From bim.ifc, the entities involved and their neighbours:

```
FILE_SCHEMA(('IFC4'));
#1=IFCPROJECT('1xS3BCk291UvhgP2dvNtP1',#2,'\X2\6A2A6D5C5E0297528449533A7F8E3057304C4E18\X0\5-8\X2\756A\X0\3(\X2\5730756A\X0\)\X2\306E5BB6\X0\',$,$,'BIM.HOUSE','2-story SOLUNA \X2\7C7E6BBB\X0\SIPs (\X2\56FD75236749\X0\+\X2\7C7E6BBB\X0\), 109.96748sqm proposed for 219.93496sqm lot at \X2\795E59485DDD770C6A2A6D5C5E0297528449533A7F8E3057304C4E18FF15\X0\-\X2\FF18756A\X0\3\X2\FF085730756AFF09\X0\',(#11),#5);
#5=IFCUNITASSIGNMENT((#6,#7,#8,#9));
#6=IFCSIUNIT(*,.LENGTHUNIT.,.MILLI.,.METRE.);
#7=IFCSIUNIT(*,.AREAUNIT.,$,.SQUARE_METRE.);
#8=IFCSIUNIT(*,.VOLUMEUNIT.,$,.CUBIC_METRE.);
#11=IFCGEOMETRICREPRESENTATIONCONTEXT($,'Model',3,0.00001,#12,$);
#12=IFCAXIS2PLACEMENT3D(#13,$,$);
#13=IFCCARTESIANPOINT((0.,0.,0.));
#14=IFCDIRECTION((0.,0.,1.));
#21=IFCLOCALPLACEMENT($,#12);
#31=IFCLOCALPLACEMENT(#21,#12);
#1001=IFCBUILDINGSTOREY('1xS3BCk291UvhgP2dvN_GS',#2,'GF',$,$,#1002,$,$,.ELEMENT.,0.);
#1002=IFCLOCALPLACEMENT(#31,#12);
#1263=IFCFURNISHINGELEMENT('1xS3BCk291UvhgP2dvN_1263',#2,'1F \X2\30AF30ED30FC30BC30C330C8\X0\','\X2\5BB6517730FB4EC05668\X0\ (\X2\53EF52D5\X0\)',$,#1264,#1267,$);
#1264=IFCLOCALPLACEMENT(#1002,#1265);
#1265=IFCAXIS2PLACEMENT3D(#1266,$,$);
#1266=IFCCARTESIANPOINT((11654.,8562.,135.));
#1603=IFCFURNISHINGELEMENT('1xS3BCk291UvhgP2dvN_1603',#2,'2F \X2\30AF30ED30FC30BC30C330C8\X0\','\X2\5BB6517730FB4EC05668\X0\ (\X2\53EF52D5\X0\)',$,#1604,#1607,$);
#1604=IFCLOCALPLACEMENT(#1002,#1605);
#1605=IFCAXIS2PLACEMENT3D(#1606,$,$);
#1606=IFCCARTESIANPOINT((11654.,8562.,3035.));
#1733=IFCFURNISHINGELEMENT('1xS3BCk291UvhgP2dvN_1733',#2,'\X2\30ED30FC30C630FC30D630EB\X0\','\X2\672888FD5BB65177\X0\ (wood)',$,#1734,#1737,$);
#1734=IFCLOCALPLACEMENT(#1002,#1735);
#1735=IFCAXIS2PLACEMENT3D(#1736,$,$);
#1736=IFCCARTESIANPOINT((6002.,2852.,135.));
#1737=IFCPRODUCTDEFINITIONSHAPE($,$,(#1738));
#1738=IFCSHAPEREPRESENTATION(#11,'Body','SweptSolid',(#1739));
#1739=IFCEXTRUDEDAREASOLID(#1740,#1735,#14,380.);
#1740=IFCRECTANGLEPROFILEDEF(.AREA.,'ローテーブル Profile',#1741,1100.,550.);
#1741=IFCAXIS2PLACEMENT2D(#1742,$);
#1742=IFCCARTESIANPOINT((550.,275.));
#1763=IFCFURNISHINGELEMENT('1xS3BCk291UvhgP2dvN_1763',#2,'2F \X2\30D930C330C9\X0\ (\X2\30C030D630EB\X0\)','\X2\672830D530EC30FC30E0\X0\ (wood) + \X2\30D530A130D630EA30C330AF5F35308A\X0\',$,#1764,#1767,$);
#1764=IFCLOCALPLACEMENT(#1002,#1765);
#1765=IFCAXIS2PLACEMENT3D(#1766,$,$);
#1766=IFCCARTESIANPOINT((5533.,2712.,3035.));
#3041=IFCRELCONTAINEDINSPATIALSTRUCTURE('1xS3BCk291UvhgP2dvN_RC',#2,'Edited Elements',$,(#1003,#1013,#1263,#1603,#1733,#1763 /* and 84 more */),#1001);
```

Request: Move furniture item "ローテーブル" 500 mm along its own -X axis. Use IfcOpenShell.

```python
import ifcopenshell
import ifcopenshell.api.geometry
import ifcopenshell.util.placement
import ifcopenshell.util.unit

model = ifcopenshell.open("bim.ifc")
unit_scale = ifcopenshell.util.unit.calculate_unit_scale(model)

item = model.by_id(1733)
matrix = ifcopenshell.util.placement.get_local_placement(item.ObjectPlacement)
matrix[:3, 3] -= matrix[:3, 0] * 0.5 / unit_scale
ifcopenshell.api.geometry.edit_object_placement(model, product=item, matrix=matrix, is_si=False)

print(ifcopenshell.util.placement.get_local_placement(item.ObjectPlacement).round(3) + 0.0)

model.write("bim_rev.ifc")
```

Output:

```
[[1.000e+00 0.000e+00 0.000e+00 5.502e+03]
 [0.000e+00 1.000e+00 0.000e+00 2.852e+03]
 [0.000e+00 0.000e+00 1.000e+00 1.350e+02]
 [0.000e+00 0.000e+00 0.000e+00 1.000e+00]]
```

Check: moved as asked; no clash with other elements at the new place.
